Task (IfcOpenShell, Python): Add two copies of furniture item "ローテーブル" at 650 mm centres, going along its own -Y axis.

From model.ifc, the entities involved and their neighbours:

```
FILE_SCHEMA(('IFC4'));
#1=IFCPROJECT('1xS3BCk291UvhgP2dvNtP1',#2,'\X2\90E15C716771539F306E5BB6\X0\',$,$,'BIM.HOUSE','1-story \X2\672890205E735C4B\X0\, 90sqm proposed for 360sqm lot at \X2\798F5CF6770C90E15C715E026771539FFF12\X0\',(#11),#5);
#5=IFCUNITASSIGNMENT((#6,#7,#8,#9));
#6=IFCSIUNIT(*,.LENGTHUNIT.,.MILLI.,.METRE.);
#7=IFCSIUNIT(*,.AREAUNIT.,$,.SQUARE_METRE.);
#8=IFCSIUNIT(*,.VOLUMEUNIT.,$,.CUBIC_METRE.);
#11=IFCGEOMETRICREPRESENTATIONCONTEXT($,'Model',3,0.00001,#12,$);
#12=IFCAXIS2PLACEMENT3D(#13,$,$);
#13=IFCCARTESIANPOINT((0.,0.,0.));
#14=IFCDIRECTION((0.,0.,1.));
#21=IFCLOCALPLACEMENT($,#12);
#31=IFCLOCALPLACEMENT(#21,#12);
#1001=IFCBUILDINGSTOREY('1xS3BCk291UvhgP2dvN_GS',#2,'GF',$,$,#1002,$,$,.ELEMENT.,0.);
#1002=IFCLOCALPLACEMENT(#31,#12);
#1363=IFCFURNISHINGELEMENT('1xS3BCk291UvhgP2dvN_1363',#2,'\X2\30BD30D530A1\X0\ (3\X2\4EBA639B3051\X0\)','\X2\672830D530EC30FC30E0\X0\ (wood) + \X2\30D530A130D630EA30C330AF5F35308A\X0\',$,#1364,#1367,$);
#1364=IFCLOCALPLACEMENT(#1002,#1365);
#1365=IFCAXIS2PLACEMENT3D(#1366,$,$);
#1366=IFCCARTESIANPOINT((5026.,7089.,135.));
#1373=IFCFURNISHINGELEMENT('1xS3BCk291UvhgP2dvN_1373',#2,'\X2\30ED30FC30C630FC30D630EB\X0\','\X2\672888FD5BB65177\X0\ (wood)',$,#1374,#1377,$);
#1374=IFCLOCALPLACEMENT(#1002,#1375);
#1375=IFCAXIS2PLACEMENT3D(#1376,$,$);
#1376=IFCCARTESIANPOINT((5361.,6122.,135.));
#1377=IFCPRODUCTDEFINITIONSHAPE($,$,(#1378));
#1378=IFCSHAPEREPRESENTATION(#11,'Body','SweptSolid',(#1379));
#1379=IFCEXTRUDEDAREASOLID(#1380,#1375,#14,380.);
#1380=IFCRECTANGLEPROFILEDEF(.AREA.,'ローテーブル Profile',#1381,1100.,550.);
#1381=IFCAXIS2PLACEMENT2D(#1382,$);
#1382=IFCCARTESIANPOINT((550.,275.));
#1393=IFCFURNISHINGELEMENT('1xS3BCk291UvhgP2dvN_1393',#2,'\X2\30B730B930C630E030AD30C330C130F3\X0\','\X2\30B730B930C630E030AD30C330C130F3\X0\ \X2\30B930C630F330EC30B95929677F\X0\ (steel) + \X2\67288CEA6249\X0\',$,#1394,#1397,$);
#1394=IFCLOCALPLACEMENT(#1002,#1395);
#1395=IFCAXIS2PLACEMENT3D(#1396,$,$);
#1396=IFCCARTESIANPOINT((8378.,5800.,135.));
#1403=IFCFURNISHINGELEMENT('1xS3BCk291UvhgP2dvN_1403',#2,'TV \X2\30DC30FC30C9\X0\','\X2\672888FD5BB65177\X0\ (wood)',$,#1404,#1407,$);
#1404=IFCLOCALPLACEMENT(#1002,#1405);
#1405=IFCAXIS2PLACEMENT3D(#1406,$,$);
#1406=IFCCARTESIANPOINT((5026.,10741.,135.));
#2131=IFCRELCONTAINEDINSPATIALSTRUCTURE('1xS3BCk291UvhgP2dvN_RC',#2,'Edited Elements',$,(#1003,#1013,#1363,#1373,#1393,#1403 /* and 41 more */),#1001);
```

```python
import ifcopenshell
import ifcopenshell.api.geometry
import ifcopenshell.api.root
import ifcopenshell.util.element
import ifcopenshell.util.placement
import ifcopenshell.util.unit

model = ifcopenshell.open("model.ifc")
unit_scale = ifcopenshell.util.unit.calculate_unit_scale(model)


def reuse_history(source, copy):
    """copy_class also copies each property set's owner history, people and application; keep the originals."""
    for rel in copy.IsDefinedBy:
        if rel.is_a("IfcRelDefinesByProperties") and (history := rel.RelatingPropertyDefinition.OwnerHistory):
            rel.RelatingPropertyDefinition.OwnerHistory = source.OwnerHistory
            ifcopenshell.util.element.remove_deep2(model, history)


source = model.by_id(1373)
base = ifcopenshell.util.placement.get_local_placement(source.ObjectPlacement)
step = -base[:3, 1] * 0.65 / unit_scale

for i in range(1, 3):
    copy = ifcopenshell.api.root.copy_class(model, product=source)
    copy.Representation = ifcopenshell.util.element.copy_deep(
        model, source.Representation, exclude=["IfcGeometricRepresentationContext", "IfcRepresentationMap"]
    )
    reuse_history(source, copy)
    matrix = base.copy()
    matrix[:3, 3] += i * step
    print("added at", matrix[:3, 3].round(3) + 0.0)
    ifcopenshell.api.geometry.edit_object_placement(model, product=copy, matrix=matrix, is_si=False)

model.write("model_edited.ifc")
```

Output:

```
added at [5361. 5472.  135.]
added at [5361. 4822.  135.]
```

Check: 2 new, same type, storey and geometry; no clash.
